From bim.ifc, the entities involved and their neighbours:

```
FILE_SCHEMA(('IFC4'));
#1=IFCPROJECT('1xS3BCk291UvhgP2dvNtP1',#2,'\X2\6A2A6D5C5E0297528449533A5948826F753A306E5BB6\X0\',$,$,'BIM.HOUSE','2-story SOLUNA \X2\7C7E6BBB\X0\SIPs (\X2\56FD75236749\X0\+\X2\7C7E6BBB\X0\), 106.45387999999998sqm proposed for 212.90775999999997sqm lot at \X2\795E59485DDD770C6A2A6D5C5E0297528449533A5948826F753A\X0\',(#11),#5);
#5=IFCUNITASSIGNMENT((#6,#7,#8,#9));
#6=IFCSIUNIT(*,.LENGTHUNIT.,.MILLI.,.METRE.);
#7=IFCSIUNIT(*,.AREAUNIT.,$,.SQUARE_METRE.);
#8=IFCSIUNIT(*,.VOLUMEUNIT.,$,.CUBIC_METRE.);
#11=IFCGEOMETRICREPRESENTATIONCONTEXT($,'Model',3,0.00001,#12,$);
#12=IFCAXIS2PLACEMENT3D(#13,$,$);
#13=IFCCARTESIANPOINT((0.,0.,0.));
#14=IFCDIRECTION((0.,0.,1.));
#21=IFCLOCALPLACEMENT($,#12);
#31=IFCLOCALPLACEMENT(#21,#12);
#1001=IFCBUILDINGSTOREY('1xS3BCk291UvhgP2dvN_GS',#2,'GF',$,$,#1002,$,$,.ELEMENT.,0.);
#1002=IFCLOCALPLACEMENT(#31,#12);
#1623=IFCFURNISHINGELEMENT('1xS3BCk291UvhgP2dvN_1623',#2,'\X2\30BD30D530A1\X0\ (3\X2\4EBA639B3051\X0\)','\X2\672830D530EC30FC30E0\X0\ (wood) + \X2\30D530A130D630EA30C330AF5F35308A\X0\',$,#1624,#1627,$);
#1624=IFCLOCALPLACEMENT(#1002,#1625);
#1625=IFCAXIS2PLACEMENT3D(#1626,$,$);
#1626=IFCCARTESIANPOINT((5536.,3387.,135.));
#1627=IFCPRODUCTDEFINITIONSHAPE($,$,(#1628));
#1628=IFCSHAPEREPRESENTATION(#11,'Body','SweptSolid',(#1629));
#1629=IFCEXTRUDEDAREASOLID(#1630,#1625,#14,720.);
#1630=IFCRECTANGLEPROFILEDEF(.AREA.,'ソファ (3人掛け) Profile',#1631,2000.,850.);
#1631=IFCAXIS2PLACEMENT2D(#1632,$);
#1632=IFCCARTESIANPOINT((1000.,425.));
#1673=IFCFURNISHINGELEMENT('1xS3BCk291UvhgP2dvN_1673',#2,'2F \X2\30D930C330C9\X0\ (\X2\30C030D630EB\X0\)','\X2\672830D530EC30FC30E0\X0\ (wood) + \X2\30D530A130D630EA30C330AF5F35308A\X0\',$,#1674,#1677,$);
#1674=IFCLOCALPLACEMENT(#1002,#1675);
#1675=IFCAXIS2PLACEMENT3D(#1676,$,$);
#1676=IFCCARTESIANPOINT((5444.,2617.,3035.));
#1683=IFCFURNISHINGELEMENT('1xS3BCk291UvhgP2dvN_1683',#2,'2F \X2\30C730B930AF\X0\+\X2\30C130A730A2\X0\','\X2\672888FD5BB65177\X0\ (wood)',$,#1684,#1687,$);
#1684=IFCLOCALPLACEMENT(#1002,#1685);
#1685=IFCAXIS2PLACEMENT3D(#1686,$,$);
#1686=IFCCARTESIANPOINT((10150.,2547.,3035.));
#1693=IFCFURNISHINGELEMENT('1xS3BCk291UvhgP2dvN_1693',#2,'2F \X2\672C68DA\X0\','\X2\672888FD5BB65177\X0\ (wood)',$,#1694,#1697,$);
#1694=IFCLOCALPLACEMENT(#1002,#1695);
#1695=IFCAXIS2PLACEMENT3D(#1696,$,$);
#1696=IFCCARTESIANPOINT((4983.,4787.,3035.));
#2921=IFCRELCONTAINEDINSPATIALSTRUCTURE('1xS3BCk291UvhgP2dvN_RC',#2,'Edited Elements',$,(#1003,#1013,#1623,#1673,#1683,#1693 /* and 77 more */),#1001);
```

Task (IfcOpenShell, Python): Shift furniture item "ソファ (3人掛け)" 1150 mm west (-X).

```python
import ifcopenshell
import ifcopenshell.api.geometry
import ifcopenshell.util.placement
import ifcopenshell.util.unit

model = ifcopenshell.open("bim.ifc")
unit_scale = ifcopenshell.util.unit.calculate_unit_scale(model)

item = model.by_id(1623)
matrix = ifcopenshell.util.placement.get_local_placement(item.ObjectPlacement)
matrix[0, 3] -= 1.15 / unit_scale
ifcopenshell.api.geometry.edit_object_placement(model, product=item, matrix=matrix, is_si=False)

print(ifcopenshell.util.placement.get_local_placement(item.ObjectPlacement).round(3) + 0.0)

model.write("bim_rev.ifc")
```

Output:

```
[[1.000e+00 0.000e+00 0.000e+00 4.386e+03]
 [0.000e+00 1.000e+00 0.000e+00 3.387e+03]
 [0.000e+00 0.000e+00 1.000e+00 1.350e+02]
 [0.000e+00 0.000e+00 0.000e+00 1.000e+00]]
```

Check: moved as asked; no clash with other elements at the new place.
